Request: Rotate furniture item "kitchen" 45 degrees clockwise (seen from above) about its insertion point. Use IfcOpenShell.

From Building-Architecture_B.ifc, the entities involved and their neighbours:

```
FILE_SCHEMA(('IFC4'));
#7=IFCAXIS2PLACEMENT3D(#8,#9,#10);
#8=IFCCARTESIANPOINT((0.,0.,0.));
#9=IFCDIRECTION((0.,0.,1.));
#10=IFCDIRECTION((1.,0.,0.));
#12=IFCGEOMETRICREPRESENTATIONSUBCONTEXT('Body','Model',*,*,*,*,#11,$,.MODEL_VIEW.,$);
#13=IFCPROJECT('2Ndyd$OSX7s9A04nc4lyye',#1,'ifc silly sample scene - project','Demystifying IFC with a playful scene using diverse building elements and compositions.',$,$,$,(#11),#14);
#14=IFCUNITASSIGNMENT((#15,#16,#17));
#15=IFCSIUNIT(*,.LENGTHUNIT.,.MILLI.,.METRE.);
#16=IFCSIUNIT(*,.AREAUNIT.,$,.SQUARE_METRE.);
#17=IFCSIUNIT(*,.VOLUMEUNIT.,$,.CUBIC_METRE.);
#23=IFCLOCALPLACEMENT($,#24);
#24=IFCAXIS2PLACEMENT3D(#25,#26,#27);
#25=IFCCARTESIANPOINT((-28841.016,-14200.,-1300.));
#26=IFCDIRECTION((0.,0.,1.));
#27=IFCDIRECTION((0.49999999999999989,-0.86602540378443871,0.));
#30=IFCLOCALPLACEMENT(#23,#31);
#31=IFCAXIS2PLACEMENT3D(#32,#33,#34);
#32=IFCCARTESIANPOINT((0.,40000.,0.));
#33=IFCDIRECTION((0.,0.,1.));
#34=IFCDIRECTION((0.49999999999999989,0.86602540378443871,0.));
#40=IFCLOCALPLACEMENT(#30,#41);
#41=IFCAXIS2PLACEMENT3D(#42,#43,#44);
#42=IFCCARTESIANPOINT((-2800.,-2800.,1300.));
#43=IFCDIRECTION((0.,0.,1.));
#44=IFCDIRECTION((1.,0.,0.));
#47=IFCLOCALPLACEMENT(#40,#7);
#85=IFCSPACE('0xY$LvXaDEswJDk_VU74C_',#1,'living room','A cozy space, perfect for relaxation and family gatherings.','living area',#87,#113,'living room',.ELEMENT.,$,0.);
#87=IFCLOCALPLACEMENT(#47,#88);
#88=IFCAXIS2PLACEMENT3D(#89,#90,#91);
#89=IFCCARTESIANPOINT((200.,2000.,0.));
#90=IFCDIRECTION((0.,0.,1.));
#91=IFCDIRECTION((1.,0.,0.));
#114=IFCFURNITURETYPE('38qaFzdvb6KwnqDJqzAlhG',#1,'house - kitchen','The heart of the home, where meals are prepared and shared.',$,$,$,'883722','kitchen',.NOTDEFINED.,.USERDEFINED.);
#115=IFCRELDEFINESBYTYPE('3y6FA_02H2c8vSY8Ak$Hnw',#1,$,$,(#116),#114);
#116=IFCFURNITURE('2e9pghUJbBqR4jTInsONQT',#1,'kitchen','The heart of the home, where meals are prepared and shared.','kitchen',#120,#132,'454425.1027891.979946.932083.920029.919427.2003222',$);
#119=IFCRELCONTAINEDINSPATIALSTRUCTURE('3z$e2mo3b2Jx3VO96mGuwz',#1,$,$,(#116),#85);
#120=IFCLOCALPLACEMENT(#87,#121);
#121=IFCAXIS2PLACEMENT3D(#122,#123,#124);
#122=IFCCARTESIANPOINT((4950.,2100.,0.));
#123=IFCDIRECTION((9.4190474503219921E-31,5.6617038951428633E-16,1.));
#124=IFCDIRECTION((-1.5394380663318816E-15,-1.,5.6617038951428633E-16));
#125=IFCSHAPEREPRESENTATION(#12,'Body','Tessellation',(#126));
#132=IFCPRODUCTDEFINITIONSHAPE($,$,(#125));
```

```python
import ifcopenshell
import ifcopenshell.api.geometry
import ifcopenshell.util.placement

model = ifcopenshell.open("Building-Architecture_B.ifc")

item = model.by_guid("2e9pghUJbBqR4jTInsONQT")
matrix = ifcopenshell.util.placement.get_local_placement(item.ObjectPlacement)
matrix = matrix @ ifcopenshell.util.placement.rotation(-45, "Z")
ifcopenshell.api.geometry.edit_object_placement(model, product=item, matrix=matrix, is_si=False)

print(ifcopenshell.util.placement.get_local_placement(item.ObjectPlacement).round(3) + 0.0)

model.write("Building-Architecture_B_edited.ifc")
```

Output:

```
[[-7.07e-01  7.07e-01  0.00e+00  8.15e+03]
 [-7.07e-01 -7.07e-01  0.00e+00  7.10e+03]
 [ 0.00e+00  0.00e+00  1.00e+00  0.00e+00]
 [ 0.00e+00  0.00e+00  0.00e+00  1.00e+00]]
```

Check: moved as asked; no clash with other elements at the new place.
